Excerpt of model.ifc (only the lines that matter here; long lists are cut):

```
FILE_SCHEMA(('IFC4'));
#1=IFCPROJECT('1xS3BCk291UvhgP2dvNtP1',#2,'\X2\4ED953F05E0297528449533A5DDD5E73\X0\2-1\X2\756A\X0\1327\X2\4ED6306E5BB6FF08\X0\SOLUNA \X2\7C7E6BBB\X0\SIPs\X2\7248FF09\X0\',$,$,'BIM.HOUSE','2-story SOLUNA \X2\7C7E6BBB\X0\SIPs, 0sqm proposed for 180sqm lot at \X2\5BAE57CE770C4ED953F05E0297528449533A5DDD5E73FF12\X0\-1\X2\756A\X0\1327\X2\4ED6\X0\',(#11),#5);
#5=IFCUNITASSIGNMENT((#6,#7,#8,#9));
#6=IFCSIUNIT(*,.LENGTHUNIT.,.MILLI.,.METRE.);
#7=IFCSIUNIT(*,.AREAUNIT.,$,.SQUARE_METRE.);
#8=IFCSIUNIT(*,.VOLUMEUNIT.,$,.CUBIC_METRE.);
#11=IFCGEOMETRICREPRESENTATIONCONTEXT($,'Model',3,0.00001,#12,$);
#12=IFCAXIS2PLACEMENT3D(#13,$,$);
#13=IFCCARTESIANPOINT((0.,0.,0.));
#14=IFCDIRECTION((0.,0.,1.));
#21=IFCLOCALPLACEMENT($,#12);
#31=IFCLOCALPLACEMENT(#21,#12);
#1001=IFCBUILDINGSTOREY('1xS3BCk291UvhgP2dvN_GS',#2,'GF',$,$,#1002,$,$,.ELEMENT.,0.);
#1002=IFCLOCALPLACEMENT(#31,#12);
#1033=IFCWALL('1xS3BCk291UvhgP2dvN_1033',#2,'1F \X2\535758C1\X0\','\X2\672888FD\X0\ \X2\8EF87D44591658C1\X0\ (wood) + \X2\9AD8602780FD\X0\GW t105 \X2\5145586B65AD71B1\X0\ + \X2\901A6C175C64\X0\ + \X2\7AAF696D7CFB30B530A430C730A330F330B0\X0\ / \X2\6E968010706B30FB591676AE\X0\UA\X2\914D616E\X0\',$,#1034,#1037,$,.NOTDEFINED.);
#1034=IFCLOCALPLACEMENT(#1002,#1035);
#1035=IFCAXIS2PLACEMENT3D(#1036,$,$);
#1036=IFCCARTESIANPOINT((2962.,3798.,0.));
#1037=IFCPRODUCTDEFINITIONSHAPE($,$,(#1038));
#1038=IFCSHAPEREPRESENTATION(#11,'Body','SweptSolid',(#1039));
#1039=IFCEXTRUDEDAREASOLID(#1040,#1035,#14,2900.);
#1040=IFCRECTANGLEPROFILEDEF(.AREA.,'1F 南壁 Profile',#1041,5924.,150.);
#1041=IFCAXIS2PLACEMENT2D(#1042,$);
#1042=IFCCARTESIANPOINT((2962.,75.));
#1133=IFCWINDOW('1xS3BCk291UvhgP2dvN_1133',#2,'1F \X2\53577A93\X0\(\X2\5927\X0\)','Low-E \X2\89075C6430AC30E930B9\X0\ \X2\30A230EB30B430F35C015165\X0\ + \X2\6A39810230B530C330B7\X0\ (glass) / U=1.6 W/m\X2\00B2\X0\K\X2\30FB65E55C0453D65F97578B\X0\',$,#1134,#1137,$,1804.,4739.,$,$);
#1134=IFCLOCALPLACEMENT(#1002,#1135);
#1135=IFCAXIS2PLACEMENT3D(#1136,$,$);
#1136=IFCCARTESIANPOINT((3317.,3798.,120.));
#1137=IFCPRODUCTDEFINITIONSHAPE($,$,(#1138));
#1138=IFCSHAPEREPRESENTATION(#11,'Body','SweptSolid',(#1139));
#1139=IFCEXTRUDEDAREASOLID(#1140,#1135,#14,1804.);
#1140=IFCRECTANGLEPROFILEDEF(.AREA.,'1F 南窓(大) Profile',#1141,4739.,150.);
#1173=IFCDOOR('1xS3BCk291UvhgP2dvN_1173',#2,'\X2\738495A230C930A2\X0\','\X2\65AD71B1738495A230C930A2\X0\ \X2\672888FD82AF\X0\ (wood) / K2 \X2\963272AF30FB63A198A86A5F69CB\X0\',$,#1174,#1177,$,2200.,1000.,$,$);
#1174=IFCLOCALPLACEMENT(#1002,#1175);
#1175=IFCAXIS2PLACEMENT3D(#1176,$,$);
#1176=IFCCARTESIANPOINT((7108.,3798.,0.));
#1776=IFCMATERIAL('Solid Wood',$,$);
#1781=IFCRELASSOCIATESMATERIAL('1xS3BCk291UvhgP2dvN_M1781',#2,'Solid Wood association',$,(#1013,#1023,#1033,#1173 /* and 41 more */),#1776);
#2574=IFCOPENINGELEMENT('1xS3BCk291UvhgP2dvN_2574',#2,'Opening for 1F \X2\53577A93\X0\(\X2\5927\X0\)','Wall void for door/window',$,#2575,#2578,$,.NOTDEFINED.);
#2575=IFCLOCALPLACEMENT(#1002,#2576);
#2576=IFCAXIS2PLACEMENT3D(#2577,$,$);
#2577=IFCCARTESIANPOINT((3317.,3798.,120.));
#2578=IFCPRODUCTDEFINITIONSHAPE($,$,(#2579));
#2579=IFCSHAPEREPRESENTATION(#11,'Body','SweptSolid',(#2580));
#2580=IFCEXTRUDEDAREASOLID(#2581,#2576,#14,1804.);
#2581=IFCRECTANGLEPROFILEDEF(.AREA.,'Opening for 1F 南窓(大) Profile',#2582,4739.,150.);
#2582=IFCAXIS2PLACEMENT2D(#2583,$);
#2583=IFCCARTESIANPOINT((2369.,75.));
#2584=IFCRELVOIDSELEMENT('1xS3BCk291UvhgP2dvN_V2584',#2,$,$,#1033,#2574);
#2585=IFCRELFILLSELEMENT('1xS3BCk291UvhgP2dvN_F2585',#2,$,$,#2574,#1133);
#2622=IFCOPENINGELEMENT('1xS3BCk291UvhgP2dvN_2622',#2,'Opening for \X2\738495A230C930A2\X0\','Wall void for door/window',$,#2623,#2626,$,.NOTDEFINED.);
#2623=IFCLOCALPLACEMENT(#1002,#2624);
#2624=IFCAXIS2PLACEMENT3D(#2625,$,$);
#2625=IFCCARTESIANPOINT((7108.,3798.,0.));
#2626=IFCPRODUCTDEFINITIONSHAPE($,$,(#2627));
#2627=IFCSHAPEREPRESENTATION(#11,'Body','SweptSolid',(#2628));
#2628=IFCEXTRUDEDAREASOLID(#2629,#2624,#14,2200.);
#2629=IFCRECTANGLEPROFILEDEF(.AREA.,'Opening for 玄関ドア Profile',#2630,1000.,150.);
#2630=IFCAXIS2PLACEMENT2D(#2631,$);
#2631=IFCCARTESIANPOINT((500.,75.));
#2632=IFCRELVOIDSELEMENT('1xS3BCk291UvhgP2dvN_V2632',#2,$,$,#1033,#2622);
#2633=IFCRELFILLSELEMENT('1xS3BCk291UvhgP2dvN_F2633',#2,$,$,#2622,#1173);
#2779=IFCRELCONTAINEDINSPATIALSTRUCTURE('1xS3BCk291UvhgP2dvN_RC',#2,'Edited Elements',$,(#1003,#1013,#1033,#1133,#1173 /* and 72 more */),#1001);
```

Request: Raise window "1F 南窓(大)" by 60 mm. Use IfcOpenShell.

```python
import numpy as np
import ifcopenshell
import ifcopenshell.api.geometry
import ifcopenshell.util.placement
import ifcopenshell.util.unit

model = ifcopenshell.open("model.ifc")
unit_scale = ifcopenshell.util.unit.calculate_unit_scale(model)

window = model.by_guid("1xS3BCk291UvhgP2dvN_1133")
opening = window.FillsVoids[0].RelatingOpeningElement
dz = 60.0

shift = np.array([0.0, 0.0, dz])
# The window is not placed relative to its opening, so move both.
for product in (opening, window):
    matrix = ifcopenshell.util.placement.get_local_placement(product.ObjectPlacement)
    matrix[:3, 3] += shift
    ifcopenshell.api.geometry.edit_object_placement(model, product=product, matrix=matrix, is_si=False)

print(f"moved by {dz * unit_scale:+.3f} m")

model.write("model_updated.ifc")
```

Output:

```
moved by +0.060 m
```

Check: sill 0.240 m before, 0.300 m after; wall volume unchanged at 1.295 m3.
